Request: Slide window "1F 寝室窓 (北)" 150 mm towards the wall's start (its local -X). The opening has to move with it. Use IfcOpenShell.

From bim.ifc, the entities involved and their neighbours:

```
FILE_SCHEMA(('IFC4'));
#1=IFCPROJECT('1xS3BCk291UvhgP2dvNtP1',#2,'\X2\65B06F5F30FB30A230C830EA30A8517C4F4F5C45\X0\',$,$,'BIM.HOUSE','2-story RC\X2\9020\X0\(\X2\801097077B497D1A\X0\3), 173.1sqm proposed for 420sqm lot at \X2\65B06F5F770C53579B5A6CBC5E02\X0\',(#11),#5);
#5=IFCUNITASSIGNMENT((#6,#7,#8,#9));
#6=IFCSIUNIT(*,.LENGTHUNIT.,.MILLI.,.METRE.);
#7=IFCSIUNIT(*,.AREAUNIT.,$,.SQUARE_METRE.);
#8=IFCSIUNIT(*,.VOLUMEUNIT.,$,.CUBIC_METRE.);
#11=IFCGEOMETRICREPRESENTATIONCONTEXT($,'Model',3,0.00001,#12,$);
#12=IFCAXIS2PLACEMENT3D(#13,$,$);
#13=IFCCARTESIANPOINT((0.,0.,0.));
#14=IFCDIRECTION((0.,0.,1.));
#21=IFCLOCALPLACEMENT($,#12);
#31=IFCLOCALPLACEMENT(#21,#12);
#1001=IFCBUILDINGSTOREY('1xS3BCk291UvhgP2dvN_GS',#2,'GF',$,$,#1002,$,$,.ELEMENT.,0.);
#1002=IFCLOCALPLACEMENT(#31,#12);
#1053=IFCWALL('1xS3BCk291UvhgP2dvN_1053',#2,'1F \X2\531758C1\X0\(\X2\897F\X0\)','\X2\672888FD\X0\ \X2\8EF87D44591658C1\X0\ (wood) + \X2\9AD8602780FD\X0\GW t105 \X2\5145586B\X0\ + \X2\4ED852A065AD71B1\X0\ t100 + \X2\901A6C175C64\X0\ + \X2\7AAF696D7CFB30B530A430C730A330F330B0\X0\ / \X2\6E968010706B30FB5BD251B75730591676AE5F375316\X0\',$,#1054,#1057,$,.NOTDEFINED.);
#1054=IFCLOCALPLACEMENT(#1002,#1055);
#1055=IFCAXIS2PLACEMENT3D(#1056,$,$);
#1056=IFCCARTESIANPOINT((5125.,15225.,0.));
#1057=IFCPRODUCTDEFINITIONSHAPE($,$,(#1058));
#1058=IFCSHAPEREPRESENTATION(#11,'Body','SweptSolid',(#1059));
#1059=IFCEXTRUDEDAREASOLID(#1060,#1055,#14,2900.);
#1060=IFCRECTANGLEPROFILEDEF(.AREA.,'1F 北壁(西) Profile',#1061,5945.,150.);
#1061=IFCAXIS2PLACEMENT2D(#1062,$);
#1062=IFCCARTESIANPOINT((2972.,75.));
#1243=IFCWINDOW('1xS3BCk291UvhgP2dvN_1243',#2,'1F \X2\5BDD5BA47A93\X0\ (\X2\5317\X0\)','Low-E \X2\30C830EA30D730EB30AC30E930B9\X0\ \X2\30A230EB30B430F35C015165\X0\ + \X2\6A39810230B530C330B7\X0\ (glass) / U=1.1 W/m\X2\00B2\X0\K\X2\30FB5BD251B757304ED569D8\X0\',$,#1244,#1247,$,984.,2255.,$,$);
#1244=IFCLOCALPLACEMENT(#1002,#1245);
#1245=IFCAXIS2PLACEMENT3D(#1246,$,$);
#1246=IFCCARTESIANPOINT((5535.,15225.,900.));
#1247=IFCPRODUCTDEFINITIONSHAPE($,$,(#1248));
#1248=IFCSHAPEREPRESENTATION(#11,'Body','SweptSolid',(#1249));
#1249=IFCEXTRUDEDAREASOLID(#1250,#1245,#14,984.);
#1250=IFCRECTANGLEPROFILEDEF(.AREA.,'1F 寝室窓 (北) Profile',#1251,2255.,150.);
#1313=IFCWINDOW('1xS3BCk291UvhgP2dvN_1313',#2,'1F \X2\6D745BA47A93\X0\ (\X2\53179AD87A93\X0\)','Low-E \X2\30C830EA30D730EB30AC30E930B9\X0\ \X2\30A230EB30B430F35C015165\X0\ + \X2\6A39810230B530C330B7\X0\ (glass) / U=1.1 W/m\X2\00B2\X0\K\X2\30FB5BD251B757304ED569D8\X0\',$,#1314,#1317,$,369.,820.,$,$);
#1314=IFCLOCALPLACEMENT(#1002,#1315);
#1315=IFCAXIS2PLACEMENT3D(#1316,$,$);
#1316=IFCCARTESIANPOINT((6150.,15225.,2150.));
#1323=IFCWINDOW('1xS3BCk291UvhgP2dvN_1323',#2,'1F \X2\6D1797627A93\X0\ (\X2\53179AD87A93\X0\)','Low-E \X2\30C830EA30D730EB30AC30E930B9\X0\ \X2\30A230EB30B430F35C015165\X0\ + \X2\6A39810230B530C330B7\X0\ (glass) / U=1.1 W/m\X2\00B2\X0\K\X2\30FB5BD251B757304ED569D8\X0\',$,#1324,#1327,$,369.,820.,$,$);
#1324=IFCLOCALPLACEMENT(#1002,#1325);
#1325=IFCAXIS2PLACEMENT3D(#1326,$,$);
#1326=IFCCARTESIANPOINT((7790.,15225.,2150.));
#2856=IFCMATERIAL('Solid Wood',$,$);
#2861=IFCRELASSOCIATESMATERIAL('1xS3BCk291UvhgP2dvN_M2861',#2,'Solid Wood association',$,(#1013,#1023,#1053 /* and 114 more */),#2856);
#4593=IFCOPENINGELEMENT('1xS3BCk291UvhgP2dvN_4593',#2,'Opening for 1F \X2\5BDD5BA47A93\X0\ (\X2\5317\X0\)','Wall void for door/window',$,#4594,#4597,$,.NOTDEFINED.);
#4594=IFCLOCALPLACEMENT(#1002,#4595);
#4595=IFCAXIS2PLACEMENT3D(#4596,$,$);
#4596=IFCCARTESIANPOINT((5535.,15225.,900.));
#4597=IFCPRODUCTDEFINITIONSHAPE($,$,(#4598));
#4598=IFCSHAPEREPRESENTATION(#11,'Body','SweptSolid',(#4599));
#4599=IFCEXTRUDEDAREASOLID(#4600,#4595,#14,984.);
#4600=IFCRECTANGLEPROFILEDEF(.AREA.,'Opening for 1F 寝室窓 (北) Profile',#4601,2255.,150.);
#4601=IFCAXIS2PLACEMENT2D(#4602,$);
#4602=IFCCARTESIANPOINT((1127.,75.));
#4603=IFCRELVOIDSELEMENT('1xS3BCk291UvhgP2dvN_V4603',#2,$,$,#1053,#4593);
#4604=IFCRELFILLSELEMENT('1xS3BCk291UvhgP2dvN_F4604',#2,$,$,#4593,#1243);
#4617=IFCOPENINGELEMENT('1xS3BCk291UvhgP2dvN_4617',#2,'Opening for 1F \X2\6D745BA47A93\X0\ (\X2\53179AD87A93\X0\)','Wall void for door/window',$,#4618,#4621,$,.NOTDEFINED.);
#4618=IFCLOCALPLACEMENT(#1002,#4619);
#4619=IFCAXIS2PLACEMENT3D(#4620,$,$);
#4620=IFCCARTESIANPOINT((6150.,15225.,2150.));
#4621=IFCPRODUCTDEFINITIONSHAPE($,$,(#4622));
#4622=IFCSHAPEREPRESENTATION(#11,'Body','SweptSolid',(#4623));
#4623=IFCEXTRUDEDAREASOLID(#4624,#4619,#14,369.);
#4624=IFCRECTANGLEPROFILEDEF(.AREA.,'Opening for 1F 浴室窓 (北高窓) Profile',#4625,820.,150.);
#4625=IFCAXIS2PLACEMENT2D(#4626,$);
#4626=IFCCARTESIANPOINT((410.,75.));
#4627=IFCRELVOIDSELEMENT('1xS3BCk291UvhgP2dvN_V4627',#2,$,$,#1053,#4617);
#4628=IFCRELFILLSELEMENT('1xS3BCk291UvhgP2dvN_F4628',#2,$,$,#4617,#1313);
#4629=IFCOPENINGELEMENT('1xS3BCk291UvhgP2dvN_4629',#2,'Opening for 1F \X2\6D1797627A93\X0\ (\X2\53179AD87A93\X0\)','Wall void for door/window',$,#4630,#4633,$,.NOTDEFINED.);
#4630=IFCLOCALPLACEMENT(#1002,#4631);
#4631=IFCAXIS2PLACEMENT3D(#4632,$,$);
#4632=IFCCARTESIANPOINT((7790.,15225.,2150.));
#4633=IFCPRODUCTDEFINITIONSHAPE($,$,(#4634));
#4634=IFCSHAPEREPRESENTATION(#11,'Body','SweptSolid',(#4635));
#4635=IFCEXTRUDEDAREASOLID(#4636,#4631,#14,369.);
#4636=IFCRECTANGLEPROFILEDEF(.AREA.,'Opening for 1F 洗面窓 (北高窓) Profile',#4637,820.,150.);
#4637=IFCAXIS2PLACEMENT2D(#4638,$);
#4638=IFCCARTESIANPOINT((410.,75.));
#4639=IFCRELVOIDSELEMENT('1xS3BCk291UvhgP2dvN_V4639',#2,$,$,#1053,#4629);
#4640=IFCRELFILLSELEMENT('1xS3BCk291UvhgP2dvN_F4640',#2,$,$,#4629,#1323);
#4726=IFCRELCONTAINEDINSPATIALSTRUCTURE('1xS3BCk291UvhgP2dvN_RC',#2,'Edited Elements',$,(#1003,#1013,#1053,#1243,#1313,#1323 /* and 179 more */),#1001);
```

```python
import ifcopenshell
import ifcopenshell.api.geometry
import ifcopenshell.util.placement

model = ifcopenshell.open("bim.ifc")

window = model.by_guid("1xS3BCk291UvhgP2dvN_1243")
opening = window.FillsVoids[0].RelatingOpeningElement
wall = opening.VoidsElements[0].RelatingBuildingElement

wall_matrix = ifcopenshell.util.placement.get_local_placement(wall.ObjectPlacement)
shift = wall_matrix[:3, 0] * -150.0
before = ifcopenshell.util.placement.get_local_placement(window.ObjectPlacement)[:3, 3].copy()

# The window is not placed relative to its opening, so move both.
for product in (opening, window):
    matrix = ifcopenshell.util.placement.get_local_placement(product.ObjectPlacement)
    matrix[:3, 3] += shift
    ifcopenshell.api.geometry.edit_object_placement(model, product=product, matrix=matrix, is_si=False)

after = ifcopenshell.util.placement.get_local_placement(window.ObjectPlacement)[:3, 3]
print("window moved by", (after - before).round(3) + 0.0)

model.write("bim-out.ifc")
```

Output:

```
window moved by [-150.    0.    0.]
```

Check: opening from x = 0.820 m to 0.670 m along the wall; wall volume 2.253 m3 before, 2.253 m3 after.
